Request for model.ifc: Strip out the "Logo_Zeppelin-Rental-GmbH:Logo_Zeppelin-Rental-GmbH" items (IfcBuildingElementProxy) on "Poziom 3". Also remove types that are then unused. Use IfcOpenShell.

First a look at what the model holds.

```python
import ifcopenshell
import ifcopenshell.util.element

model = ifcopenshell.open("model.ifc")
print(model.schema)
storey = next(s for s in model.by_type("IfcBuildingStorey") if s.Name == "Poziom 3")
proxies = [e for e in ifcopenshell.util.element.get_decomposition(storey) if e.is_a("IfcBuildingElementProxy")]
seen = {}
for e in proxies:
    element_type = ifcopenshell.util.element.get_type(e)
    name = element_type.Name if element_type not in (None, e) else None
    seen[name] = seen.get(name, 0) + 1
for name, count in sorted(seen.items(), key=str):
    print(count, "x", name)
```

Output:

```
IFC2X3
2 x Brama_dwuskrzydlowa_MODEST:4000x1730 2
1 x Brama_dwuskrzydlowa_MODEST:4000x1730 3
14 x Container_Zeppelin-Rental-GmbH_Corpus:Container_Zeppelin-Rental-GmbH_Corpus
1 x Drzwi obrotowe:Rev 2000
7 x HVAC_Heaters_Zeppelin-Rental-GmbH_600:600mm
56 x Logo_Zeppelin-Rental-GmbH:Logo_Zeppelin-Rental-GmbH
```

```python
import ifcopenshell
import ifcopenshell.api.root
import ifcopenshell.util.element

model = ifcopenshell.open("model.ifc")

storey = next(s for s in model.by_type("IfcBuildingStorey") if s.Name == "Poziom 3")
proxies = [e for e in ifcopenshell.util.element.get_decomposition(storey) if e.is_a("IfcBuildingElementProxy")]
targets = [e for e in proxies if (t := ifcopenshell.util.element.get_type(e)) not in (None, e) and t.Name == "Logo_Zeppelin-Rental-GmbH:Logo_Zeppelin-Rental-GmbH"]
types = {ifcopenshell.util.element.get_type(e) for e in targets} - {None, *targets}

for e in targets:
    ifcopenshell.api.root.remove_product(model, product=e)
print(len(targets), "removed")

unused = [t for t in types if not ifcopenshell.util.element.get_types(t)]
for t in unused:
    ifcopenshell.api.root.remove_product(model, product=t)
print(len(unused), "unused types removed")

model.write("model_rev.ifc")
```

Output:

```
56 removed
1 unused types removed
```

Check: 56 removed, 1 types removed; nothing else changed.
